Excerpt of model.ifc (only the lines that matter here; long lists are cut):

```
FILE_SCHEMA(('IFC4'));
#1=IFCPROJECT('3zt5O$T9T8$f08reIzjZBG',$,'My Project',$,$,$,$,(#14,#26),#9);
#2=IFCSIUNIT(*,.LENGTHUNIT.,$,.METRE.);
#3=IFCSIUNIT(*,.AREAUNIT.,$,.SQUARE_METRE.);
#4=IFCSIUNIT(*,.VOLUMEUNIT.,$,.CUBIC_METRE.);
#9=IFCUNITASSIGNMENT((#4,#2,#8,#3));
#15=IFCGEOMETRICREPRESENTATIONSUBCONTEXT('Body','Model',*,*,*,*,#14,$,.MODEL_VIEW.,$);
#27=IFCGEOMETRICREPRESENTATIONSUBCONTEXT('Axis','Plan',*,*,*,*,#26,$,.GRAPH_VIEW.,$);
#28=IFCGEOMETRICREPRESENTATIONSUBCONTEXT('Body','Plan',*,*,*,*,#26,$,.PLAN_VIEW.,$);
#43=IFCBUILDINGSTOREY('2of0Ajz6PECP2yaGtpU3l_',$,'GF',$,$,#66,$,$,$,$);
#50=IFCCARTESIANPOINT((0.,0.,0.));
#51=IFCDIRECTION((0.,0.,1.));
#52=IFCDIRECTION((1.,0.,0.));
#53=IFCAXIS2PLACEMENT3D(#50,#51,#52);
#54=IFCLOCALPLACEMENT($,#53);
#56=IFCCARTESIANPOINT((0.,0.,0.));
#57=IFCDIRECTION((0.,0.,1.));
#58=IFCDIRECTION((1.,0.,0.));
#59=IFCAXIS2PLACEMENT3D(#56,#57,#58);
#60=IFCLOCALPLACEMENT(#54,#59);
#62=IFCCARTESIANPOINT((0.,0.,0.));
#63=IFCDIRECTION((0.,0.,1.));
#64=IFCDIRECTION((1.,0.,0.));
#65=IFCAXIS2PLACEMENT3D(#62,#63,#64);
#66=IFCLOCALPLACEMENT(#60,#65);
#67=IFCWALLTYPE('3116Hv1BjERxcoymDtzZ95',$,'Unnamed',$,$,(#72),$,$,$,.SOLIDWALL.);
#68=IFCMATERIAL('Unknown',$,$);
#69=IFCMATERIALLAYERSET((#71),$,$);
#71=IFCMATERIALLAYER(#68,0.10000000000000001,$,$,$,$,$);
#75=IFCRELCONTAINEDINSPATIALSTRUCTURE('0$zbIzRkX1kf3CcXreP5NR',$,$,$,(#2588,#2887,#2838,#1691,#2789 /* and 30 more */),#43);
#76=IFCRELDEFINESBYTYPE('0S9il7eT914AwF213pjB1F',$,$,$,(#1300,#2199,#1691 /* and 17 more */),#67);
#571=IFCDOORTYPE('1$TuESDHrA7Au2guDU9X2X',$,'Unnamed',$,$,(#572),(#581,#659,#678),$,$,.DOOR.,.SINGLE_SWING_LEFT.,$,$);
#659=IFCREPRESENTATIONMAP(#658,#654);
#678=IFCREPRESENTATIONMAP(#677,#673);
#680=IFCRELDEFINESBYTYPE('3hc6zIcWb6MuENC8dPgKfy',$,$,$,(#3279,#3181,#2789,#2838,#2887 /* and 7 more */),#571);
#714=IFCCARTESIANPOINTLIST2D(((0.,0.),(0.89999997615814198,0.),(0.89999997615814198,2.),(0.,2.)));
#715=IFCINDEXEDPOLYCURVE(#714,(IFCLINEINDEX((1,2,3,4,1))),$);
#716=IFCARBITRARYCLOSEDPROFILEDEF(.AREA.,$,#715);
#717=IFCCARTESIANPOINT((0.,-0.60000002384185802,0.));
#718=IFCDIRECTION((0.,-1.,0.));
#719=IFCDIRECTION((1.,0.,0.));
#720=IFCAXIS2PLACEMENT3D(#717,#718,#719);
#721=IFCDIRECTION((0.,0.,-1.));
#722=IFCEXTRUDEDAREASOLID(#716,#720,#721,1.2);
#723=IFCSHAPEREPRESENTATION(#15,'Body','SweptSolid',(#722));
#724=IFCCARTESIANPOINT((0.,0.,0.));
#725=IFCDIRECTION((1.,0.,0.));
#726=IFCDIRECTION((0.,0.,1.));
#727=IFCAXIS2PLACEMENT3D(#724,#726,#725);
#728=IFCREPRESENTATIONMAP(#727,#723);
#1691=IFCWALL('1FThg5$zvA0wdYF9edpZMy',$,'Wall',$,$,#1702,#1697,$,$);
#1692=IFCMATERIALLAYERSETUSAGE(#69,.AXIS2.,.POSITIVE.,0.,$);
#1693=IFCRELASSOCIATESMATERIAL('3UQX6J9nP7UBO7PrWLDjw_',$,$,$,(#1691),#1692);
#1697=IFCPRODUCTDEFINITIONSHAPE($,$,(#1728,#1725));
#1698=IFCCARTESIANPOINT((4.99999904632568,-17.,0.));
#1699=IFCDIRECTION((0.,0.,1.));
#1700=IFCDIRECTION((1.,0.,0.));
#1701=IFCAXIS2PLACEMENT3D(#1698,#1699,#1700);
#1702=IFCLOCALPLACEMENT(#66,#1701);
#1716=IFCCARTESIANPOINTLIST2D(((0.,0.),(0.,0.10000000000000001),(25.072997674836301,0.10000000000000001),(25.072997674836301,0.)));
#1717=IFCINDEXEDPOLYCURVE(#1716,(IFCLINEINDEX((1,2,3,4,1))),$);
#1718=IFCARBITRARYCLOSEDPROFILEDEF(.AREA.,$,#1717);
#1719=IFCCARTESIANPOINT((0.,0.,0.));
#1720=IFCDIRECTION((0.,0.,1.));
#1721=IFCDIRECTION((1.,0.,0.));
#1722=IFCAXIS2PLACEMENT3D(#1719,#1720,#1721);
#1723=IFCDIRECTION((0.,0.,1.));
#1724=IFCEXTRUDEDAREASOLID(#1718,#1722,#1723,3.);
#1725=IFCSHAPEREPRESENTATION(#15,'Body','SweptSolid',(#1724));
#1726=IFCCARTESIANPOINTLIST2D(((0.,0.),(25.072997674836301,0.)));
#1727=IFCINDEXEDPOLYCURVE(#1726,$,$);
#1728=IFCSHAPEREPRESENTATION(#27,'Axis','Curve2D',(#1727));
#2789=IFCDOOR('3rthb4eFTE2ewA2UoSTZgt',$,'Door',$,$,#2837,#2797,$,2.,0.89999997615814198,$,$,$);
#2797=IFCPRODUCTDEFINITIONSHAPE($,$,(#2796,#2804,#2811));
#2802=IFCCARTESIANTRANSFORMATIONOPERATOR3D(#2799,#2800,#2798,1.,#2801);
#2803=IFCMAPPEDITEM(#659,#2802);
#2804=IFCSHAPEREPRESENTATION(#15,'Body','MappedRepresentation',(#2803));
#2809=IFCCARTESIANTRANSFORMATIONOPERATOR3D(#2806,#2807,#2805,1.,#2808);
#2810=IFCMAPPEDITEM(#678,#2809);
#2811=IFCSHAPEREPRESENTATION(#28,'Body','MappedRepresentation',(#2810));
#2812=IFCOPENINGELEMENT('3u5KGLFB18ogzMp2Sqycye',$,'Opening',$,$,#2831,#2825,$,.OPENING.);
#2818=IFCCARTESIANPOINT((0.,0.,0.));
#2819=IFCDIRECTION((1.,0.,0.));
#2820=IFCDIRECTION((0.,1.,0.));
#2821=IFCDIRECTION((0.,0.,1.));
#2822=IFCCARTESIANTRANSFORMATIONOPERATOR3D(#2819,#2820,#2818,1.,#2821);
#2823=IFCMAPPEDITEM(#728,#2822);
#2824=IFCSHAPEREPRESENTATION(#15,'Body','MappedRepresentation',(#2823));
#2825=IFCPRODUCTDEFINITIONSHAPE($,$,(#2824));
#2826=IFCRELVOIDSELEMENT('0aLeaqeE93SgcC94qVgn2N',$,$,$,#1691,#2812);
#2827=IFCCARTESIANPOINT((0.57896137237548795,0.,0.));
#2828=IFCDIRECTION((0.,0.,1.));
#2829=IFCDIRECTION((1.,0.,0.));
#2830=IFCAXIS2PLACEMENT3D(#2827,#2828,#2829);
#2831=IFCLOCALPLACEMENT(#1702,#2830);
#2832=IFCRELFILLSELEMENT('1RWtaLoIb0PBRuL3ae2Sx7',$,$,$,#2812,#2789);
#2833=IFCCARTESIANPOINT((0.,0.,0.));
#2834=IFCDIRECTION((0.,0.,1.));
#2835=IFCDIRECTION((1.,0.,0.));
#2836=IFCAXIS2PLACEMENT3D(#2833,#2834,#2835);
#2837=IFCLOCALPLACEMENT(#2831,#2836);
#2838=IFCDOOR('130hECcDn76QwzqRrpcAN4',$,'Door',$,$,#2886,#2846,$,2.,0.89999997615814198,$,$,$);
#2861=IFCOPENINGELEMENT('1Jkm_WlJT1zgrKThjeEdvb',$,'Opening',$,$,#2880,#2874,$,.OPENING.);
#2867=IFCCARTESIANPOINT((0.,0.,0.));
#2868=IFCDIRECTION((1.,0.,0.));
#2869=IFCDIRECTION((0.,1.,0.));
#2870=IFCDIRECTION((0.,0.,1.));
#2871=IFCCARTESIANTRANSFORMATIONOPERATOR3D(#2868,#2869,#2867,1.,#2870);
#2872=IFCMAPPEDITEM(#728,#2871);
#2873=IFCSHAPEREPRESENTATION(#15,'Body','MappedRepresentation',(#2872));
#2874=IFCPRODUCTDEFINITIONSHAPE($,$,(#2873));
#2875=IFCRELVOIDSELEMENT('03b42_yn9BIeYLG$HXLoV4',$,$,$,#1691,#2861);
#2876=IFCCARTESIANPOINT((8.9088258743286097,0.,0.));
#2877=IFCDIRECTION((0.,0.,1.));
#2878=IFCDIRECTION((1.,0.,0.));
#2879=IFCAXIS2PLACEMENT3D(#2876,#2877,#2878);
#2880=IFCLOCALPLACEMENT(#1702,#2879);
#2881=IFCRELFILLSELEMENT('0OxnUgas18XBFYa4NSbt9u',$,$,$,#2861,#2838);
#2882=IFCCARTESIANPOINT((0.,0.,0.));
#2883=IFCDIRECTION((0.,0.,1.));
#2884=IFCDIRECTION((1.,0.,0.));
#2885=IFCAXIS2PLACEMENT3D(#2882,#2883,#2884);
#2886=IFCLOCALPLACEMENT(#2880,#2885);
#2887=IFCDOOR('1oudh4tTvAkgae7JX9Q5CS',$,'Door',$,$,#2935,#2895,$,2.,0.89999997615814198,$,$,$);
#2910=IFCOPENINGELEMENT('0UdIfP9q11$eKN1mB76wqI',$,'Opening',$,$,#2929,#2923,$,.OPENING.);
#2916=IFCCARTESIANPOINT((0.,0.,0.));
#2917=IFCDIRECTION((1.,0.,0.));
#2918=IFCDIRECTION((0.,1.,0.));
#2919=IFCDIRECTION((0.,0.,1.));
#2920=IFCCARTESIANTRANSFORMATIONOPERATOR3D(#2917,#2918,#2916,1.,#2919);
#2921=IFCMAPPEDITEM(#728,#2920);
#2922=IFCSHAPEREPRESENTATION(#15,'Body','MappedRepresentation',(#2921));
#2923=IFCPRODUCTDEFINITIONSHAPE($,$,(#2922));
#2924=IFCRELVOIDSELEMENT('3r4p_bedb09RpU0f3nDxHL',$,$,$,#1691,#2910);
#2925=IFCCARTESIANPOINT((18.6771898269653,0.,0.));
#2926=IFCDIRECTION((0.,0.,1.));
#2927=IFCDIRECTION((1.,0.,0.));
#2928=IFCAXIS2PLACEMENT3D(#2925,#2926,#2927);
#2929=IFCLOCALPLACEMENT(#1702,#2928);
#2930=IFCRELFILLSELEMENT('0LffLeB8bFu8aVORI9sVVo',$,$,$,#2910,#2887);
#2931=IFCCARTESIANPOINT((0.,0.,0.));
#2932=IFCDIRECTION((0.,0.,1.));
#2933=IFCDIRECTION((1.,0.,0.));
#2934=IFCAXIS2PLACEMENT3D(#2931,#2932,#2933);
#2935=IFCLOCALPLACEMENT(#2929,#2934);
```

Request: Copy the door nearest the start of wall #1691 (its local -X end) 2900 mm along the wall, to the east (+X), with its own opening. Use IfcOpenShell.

```python
import ifcopenshell
import ifcopenshell.api.feature
import ifcopenshell.api.geometry
import ifcopenshell.api.root
import ifcopenshell.geom
import ifcopenshell.util.element
import ifcopenshell.util.placement
import ifcopenshell.util.shape
import ifcopenshell.util.unit

model = ifcopenshell.open("model.ifc")
unit_scale = ifcopenshell.util.unit.calculate_unit_scale(model)
settings = ifcopenshell.geom.settings()


def volume(element):
    """Net volume in cubic metres, openings subtracted."""
    shape = ifcopenshell.geom.create_shape(settings, element)
    return ifcopenshell.util.shape.get_volume(shape.geometry)


door = model.by_guid("3rthb4eFTE2ewA2UoSTZgt")
opening = door.FillsVoids[0].RelatingOpeningElement
wall = opening.VoidsElements[0].RelatingBuildingElement
before = volume(wall)
shift = ifcopenshell.util.placement.get_local_placement(wall.ObjectPlacement)[:3, 0] * 2.9 / unit_scale

# copy_class copies the void relationship, type, container and properties, but no geometry.
new_opening = ifcopenshell.api.root.copy_class(model, product=opening)
new_opening.Representation = ifcopenshell.util.element.copy_deep(
    model, opening.Representation, exclude=["IfcGeometricRepresentationContext", "IfcRepresentationMap"]
)
new_door = ifcopenshell.api.root.copy_class(model, product=door)
new_door.Representation = ifcopenshell.util.element.copy_deep(
    model, door.Representation, exclude=["IfcGeometricRepresentationContext", "IfcRepresentationMap"]
)
ifcopenshell.api.feature.add_filling(model, opening=new_opening, element=new_door)

for old, new in ((opening, new_opening), (door, new_door)):
    matrix = ifcopenshell.util.placement.get_local_placement(old.ObjectPlacement)
    matrix[:3, 3] += shift
    ifcopenshell.api.geometry.edit_object_placement(model, product=new, matrix=matrix, is_si=False)

after = volume(wall)

print(f"wall volume {before:.3f} -> {after:.3f} m3")

model.write("model_v2.ifc")
```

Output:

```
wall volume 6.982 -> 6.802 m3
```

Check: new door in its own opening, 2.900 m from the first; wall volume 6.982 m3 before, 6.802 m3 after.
